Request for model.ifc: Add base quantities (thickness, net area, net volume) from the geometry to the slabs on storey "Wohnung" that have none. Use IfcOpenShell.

First a look at what the model holds.

```python
import ifcopenshell
import ifcopenshell.util.element
import ifcopenshell.util.unit

model = ifcopenshell.open("model.ifc")
print(model.schema)
for unit_type in ("LENGTHUNIT", "AREAUNIT", "VOLUMEUNIT"):
    print(unit_type, ifcopenshell.util.unit.calculate_unit_scale(model, unit_type))
storey = next(s for s in model.by_type("IfcBuildingStorey") if s.Name == "Wohnung")
slabs = [e for e in ifcopenshell.util.element.get_decomposition(storey) if e.is_a("IfcSlab")]
for e in sorted(slabs, key=lambda e: e.id()):
    print(e.id(), e.is_a(), e.Name, list(ifcopenshell.util.element.get_psets(e, qtos_only=True)), sep=" | ")
```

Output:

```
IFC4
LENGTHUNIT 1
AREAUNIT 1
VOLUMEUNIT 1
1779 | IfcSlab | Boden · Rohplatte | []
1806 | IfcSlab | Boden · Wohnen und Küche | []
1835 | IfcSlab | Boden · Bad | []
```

```python
import ifcopenshell
import ifcopenshell.api.pset
import ifcopenshell.geom
import ifcopenshell.util.element
import ifcopenshell.util.shape
import ifcopenshell.util.unit

model = ifcopenshell.open("model.ifc")
unit_scale = ifcopenshell.util.unit.calculate_unit_scale(model)
area_scale = ifcopenshell.util.unit.calculate_unit_scale(model, "AREAUNIT")
volume_scale = ifcopenshell.util.unit.calculate_unit_scale(model, "VOLUMEUNIT")
settings = ifcopenshell.geom.settings()

storey = next(s for s in model.by_type("IfcBuildingStorey") if s.Name == "Wohnung")
slabs = [e for e in ifcopenshell.util.element.get_decomposition(storey) if e.is_a("IfcSlab")]

for e in sorted(slabs, key=lambda e: e.id()):
    if ifcopenshell.util.element.get_psets(e, qtos_only=True, should_inherit=False):
        continue
    # Geometry comes back in metres, in the element's own axes.
    shape = ifcopenshell.geom.create_shape(settings, e)
    values = {
        "Width": ifcopenshell.util.shape.get_z(shape.geometry) / unit_scale,
        "NetArea": ifcopenshell.util.shape.get_footprint_area(shape.geometry) / area_scale,
        "NetVolume": ifcopenshell.util.shape.get_volume(shape.geometry) / volume_scale,
    }
    qto = ifcopenshell.api.pset.add_qto(model, product=e, name="Qto_SlabBaseQuantities")
    ifcopenshell.api.pset.edit_qto(model, qto=qto, properties=values)
    print(e.id(), {k: round(v, 3) for k, v in values.items()})

model.write("model_updated.ifc")
```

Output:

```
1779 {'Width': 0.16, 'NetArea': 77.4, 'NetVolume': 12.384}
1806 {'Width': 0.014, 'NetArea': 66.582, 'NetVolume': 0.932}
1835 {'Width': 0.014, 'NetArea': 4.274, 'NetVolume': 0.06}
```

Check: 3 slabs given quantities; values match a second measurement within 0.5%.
